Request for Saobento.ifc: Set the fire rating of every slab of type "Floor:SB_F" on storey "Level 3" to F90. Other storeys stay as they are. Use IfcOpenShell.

First a look at what the model holds.

```python
import ifcopenshell
import ifcopenshell.util.element

model = ifcopenshell.open("Saobento.ifc")
print(model.schema)
storey = next(s for s in model.by_type("IfcBuildingStorey") if s.Name == "Level 3")
slabs = [e for e in ifcopenshell.util.element.get_decomposition(storey) if e.is_a("IfcSlab")]
seen = {}
for e in slabs:
    element_type = ifcopenshell.util.element.get_type(e)
    key = (element_type.Name if element_type != e and element_type else None, ifcopenshell.util.element.get_pset(e, "Pset_SlabCommon", "FireRating"))
    seen[key] = seen.get(key, 0) + 1
for (name, value), count in sorted(seen.items(), key=str):
    print(count, "x", name, "|", value)
```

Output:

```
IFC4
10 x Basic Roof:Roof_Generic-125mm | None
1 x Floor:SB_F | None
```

```python
import ifcopenshell
import ifcopenshell.api.pset
import ifcopenshell.util.element

model = ifcopenshell.open("Saobento.ifc")

storey = next(s for s in model.by_type("IfcBuildingStorey") if s.Name == "Level 3")
slabs = [e for e in ifcopenshell.util.element.get_decomposition(storey) if e.is_a("IfcSlab")]

count = 0
for e in slabs:
    element_type = ifcopenshell.util.element.get_type(e)
    if element_type in (None, e) or element_type.Name != "Floor:SB_F":
        continue
    # add_pset returns the element's existing set when there is one.
    pset = ifcopenshell.api.pset.add_pset(model, product=e, name="Pset_SlabCommon")
    ifcopenshell.api.pset.edit_pset(model, pset=pset, properties={"FireRating": "F90"})
    count += 1

print(count, "slabs updated")

model.write("Saobento_edited.ifc")
```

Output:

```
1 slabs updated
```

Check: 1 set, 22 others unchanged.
